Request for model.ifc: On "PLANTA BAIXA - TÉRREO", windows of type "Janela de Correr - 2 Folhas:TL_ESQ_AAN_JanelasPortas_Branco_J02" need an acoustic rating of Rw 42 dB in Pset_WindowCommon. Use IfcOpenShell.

First a look at what the model holds.

```python
import ifcopenshell
import ifcopenshell.util.element

model = ifcopenshell.open("model.ifc")
print(model.schema)
storey = next(s for s in model.by_type("IfcBuildingStorey") if s.Name == "PLANTA BAIXA - TÉRREO")
windows = [e for e in ifcopenshell.util.element.get_decomposition(storey) if e.is_a("IfcWindow")]
seen = {}
for e in windows:
    element_type = ifcopenshell.util.element.get_type(e)
    key = (element_type.Name if element_type != e and element_type else None, ifcopenshell.util.element.get_pset(e, "Pset_WindowCommon", "AcousticRating"))
    seen[key] = seen.get(key, 0) + 1
for (name, value), count in sorted(seen.items(), key=str):
    print(count, "x", name, "|", value)
```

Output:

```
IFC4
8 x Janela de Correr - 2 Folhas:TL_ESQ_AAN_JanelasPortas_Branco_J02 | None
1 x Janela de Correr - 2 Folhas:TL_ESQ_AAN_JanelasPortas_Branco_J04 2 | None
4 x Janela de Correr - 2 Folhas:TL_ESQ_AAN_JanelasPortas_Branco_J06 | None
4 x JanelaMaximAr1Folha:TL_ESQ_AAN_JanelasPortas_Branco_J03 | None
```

```python
import ifcopenshell
import ifcopenshell.api.pset
import ifcopenshell.util.element

model = ifcopenshell.open("model.ifc")

storey = next(s for s in model.by_type("IfcBuildingStorey") if s.Name == "PLANTA BAIXA - TÉRREO")
windows = [e for e in ifcopenshell.util.element.get_decomposition(storey) if e.is_a("IfcWindow")]

count = 0
for e in windows:
    element_type = ifcopenshell.util.element.get_type(e)
    if element_type in (None, e) or element_type.Name != "Janela de Correr - 2 Folhas:TL_ESQ_AAN_JanelasPortas_Branco_J02":
        continue
    # add_pset returns the element's existing set when there is one.
    pset = ifcopenshell.api.pset.add_pset(model, product=e, name="Pset_WindowCommon")
    ifcopenshell.api.pset.edit_pset(model, pset=pset, properties={"AcousticRating": "Rw 42 dB"})
    count += 1

print(count, "windows updated")

model.write("model_v2.ifc")
```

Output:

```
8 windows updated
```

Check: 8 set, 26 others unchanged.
